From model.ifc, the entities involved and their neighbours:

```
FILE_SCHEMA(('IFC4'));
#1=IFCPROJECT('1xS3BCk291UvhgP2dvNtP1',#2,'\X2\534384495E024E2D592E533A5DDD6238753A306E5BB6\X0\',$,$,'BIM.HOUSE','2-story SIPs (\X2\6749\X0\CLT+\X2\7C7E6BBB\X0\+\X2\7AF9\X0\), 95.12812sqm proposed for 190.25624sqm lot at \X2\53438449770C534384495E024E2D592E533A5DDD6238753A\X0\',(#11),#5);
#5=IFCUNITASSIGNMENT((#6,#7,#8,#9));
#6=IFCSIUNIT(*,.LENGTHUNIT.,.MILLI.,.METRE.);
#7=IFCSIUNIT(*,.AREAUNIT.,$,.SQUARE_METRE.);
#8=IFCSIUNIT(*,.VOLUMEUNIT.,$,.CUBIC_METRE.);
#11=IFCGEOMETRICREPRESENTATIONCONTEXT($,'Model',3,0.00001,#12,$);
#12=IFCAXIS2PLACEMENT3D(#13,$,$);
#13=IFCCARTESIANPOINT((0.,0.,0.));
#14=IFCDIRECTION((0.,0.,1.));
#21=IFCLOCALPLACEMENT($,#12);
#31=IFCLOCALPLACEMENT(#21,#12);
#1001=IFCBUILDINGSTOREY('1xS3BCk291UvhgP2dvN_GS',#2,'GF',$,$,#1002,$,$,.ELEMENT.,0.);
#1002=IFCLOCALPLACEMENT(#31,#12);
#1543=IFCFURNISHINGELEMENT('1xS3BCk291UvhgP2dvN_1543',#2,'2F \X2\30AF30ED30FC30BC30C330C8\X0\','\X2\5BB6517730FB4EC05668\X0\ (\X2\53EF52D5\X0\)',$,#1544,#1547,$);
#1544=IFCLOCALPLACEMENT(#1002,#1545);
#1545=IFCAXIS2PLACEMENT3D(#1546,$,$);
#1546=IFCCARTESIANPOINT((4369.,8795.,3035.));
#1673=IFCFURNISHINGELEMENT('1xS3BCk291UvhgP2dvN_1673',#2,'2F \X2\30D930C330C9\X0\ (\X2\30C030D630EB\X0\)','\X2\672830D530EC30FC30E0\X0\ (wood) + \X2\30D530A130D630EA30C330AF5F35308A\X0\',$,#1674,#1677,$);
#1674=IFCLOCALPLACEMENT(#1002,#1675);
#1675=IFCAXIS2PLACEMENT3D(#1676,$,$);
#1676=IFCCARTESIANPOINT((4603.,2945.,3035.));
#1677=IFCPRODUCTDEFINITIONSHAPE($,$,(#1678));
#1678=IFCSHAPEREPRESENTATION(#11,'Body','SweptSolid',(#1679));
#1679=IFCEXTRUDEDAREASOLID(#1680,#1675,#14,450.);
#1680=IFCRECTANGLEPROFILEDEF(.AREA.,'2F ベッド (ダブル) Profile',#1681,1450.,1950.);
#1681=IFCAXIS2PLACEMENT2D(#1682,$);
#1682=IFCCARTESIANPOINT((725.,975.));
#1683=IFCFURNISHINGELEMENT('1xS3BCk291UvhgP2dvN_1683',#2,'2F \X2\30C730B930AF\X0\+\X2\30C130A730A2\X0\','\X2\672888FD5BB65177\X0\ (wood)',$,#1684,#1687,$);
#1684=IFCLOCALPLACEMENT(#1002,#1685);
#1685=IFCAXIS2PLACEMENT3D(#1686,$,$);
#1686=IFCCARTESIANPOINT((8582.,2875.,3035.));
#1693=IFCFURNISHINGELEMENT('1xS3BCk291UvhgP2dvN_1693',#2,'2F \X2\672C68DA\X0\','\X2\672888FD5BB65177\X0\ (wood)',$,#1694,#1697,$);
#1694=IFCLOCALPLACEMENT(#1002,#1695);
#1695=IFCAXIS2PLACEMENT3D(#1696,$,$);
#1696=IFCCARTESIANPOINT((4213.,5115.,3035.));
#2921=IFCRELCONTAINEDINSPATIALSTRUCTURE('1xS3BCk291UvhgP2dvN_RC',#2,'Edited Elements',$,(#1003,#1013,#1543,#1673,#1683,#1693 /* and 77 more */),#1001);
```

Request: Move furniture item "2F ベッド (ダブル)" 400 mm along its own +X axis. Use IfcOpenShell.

```python
import ifcopenshell
import ifcopenshell.api.geometry
import ifcopenshell.util.placement

model = ifcopenshell.open("model.ifc")

item = model.by_id(1673)
matrix = ifcopenshell.util.placement.get_local_placement(item.ObjectPlacement)
matrix[:3, 3] += matrix[:3, 0] * 400.0
ifcopenshell.api.geometry.edit_object_placement(model, product=item, matrix=matrix, is_si=False)

print(ifcopenshell.util.placement.get_local_placement(item.ObjectPlacement).round(3) + 0.0)

model.write("model_updated.ifc")
```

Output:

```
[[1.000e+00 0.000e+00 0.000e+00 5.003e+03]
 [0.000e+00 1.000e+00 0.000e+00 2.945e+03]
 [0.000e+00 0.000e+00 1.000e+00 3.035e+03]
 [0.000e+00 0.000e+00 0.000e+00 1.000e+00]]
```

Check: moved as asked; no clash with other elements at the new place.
